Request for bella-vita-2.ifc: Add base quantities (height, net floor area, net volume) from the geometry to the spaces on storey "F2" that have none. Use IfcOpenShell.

First a look at what the model holds.

```python
import ifcopenshell
import ifcopenshell.util.element
import ifcopenshell.util.unit

model = ifcopenshell.open("bella-vita-2.ifc")
print(model.schema)
for unit_type in ("LENGTHUNIT", "AREAUNIT", "VOLUMEUNIT"):
    print(unit_type, ifcopenshell.util.unit.calculate_unit_scale(model, unit_type))
storey = next(s for s in model.by_type("IfcBuildingStorey") if s.Name == "F2")
spaces = [e for e in ifcopenshell.util.element.get_decomposition(storey) if e.is_a("IfcSpace")]
for e in sorted(spaces, key=lambda e: e.id()):
    print(e.id(), e.is_a(), e.Name, list(ifcopenshell.util.element.get_psets(e, qtos_only=True)), sep=" | ")
```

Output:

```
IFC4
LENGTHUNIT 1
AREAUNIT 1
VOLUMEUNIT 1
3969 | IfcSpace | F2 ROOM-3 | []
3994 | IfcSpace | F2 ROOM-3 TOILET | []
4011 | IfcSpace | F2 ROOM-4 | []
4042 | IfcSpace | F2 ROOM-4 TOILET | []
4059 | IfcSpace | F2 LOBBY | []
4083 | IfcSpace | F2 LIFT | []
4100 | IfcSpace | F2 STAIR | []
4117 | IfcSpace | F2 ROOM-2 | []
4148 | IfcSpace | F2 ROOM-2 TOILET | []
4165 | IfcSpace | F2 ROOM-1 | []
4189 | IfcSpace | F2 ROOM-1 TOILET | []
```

```python
import ifcopenshell
import ifcopenshell.api.pset
import ifcopenshell.geom
import ifcopenshell.util.element
import ifcopenshell.util.shape
import ifcopenshell.util.unit

model = ifcopenshell.open("bella-vita-2.ifc")
unit_scale = ifcopenshell.util.unit.calculate_unit_scale(model)
area_scale = ifcopenshell.util.unit.calculate_unit_scale(model, "AREAUNIT")
volume_scale = ifcopenshell.util.unit.calculate_unit_scale(model, "VOLUMEUNIT")
settings = ifcopenshell.geom.settings()

storey = next(s for s in model.by_type("IfcBuildingStorey") if s.Name == "F2")
spaces = [e for e in ifcopenshell.util.element.get_decomposition(storey) if e.is_a("IfcSpace")]

for e in sorted(spaces, key=lambda e: e.id()):
    if ifcopenshell.util.element.get_psets(e, qtos_only=True, should_inherit=False):
        continue
    # Geometry comes back in metres, in the element's own axes.
    shape = ifcopenshell.geom.create_shape(settings, e)
    values = {
        "Height": ifcopenshell.util.shape.get_z(shape.geometry) / unit_scale,
        "NetFloorArea": ifcopenshell.util.shape.get_footprint_area(shape.geometry) / area_scale,
        "NetVolume": ifcopenshell.util.shape.get_volume(shape.geometry) / volume_scale,
    }
    qto = ifcopenshell.api.pset.add_qto(model, product=e, name="Qto_SpaceBaseQuantities")
    ifcopenshell.api.pset.edit_qto(model, qto=qto, properties=values)
    print(e.id(), {k: round(v, 3) for k, v in values.items()})

model.write("bella-vita-2-out.ifc")
```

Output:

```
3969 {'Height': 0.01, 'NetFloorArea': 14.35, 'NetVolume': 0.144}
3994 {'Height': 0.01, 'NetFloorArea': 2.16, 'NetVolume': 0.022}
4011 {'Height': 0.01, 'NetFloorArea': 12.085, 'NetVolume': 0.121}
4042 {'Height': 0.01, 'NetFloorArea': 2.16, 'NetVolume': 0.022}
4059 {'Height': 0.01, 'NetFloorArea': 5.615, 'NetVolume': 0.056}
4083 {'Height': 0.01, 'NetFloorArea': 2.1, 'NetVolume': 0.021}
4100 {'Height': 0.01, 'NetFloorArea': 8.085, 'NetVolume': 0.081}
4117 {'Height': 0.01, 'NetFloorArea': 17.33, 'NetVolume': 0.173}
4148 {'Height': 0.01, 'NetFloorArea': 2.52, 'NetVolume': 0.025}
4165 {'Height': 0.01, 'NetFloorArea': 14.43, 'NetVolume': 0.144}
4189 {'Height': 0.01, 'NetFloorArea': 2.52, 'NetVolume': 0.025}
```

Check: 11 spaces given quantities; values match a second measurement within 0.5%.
